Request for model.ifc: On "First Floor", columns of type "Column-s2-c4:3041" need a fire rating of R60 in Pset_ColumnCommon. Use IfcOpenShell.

First a look at what the model holds.

```python
import ifcopenshell
import ifcopenshell.util.element

model = ifcopenshell.open("model.ifc")
print(model.schema)
storey = next(s for s in model.by_type("IfcBuildingStorey") if s.Name == "First Floor")
columns = [e for e in ifcopenshell.util.element.get_decomposition(storey) if e.is_a("IfcColumn")]
seen = {}
for e in columns:
    element_type = ifcopenshell.util.element.get_type(e)
    key = (element_type.Name if element_type != e and element_type else None, ifcopenshell.util.element.get_pset(e, "Pset_ColumnCommon", "FireRating"))
    seen[key] = seen.get(key, 0) + 1
for (name, value), count in sorted(seen.items(), key=str):
    print(count, "x", name, "|", value)
```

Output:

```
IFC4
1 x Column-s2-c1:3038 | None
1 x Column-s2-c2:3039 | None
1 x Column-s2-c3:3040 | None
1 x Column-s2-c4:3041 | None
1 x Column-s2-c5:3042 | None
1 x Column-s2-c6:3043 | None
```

```python
import ifcopenshell
import ifcopenshell.api.pset
import ifcopenshell.util.element

model = ifcopenshell.open("model.ifc")

storey = next(s for s in model.by_type("IfcBuildingStorey") if s.Name == "First Floor")
columns = [e for e in ifcopenshell.util.element.get_decomposition(storey) if e.is_a("IfcColumn")]

count = 0
for e in columns:
    element_type = ifcopenshell.util.element.get_type(e)
    if element_type in (None, e) or element_type.Name != "Column-s2-c4:3041":
        continue
    # add_pset returns the element's existing set when there is one.
    pset = ifcopenshell.api.pset.add_pset(model, product=e, name="Pset_ColumnCommon")
    ifcopenshell.api.pset.edit_pset(model, pset=pset, properties={"FireRating": "R60"})
    count += 1

print(count, "columns updated")

model.write("model-out.ifc")
```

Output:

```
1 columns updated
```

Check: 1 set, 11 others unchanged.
